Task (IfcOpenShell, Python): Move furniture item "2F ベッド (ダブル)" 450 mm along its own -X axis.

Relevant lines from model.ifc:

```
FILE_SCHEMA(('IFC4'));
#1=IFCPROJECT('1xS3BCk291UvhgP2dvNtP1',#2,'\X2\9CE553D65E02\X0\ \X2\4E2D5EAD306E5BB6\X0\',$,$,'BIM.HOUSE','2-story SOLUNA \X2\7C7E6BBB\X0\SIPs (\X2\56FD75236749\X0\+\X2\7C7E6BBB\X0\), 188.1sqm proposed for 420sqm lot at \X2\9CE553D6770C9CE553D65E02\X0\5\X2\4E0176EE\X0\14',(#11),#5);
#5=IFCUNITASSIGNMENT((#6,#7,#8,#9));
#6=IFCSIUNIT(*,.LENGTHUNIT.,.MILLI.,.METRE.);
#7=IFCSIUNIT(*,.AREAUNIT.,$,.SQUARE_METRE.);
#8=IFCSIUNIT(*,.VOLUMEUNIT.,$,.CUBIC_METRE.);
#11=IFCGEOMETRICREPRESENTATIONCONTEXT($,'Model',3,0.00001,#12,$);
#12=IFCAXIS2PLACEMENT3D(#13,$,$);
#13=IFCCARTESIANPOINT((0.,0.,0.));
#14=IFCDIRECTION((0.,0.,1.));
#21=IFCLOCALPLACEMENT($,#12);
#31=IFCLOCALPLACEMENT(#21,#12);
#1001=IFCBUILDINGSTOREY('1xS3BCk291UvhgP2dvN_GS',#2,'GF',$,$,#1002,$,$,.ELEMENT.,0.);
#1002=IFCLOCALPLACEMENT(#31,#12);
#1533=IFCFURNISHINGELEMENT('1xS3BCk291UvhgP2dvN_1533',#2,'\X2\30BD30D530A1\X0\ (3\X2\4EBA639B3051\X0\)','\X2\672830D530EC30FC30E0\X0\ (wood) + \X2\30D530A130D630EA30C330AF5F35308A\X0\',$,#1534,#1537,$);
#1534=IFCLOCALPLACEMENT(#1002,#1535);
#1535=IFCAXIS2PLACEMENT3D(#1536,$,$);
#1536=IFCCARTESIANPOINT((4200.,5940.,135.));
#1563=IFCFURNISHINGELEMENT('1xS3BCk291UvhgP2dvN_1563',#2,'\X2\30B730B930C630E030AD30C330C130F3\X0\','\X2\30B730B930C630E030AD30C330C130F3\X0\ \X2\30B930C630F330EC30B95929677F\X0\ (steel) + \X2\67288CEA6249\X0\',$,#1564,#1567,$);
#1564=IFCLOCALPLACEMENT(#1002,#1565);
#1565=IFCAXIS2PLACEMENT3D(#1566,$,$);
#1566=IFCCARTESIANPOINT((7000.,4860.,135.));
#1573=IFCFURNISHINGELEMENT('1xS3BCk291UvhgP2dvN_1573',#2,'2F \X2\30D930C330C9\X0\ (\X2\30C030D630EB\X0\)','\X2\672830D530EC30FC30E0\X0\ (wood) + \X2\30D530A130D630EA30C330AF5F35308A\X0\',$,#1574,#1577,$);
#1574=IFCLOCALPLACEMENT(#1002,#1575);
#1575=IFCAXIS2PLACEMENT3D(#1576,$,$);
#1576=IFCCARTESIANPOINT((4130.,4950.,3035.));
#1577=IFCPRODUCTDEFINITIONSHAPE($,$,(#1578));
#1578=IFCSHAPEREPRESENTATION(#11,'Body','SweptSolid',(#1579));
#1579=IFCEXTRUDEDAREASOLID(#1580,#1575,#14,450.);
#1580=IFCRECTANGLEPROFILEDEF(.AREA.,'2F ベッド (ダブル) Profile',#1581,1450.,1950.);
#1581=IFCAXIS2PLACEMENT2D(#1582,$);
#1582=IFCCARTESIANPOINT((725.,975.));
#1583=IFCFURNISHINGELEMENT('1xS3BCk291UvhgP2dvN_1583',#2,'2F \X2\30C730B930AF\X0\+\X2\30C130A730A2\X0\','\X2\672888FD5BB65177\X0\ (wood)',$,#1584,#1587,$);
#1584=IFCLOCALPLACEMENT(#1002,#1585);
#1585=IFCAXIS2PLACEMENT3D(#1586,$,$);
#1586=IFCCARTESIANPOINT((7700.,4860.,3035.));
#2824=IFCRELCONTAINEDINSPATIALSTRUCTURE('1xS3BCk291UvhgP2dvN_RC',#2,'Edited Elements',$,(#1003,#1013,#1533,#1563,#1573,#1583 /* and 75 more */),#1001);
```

```python
import ifcopenshell
import ifcopenshell.api.geometry
import ifcopenshell.util.placement

model = ifcopenshell.open("model.ifc")

item = model.by_id(1573)
matrix = ifcopenshell.util.placement.get_local_placement(item.ObjectPlacement)
matrix[:3, 3] -= matrix[:3, 0] * 450.0
ifcopenshell.api.geometry.edit_object_placement(model, product=item, matrix=matrix, is_si=False)

print(ifcopenshell.util.placement.get_local_placement(item.ObjectPlacement).round(3) + 0.0)

model.write("model-out.ifc")
```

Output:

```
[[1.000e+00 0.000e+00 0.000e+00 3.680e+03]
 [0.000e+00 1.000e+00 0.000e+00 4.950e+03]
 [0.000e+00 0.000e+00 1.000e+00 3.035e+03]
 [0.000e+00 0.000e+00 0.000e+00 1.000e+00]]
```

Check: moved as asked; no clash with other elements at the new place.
